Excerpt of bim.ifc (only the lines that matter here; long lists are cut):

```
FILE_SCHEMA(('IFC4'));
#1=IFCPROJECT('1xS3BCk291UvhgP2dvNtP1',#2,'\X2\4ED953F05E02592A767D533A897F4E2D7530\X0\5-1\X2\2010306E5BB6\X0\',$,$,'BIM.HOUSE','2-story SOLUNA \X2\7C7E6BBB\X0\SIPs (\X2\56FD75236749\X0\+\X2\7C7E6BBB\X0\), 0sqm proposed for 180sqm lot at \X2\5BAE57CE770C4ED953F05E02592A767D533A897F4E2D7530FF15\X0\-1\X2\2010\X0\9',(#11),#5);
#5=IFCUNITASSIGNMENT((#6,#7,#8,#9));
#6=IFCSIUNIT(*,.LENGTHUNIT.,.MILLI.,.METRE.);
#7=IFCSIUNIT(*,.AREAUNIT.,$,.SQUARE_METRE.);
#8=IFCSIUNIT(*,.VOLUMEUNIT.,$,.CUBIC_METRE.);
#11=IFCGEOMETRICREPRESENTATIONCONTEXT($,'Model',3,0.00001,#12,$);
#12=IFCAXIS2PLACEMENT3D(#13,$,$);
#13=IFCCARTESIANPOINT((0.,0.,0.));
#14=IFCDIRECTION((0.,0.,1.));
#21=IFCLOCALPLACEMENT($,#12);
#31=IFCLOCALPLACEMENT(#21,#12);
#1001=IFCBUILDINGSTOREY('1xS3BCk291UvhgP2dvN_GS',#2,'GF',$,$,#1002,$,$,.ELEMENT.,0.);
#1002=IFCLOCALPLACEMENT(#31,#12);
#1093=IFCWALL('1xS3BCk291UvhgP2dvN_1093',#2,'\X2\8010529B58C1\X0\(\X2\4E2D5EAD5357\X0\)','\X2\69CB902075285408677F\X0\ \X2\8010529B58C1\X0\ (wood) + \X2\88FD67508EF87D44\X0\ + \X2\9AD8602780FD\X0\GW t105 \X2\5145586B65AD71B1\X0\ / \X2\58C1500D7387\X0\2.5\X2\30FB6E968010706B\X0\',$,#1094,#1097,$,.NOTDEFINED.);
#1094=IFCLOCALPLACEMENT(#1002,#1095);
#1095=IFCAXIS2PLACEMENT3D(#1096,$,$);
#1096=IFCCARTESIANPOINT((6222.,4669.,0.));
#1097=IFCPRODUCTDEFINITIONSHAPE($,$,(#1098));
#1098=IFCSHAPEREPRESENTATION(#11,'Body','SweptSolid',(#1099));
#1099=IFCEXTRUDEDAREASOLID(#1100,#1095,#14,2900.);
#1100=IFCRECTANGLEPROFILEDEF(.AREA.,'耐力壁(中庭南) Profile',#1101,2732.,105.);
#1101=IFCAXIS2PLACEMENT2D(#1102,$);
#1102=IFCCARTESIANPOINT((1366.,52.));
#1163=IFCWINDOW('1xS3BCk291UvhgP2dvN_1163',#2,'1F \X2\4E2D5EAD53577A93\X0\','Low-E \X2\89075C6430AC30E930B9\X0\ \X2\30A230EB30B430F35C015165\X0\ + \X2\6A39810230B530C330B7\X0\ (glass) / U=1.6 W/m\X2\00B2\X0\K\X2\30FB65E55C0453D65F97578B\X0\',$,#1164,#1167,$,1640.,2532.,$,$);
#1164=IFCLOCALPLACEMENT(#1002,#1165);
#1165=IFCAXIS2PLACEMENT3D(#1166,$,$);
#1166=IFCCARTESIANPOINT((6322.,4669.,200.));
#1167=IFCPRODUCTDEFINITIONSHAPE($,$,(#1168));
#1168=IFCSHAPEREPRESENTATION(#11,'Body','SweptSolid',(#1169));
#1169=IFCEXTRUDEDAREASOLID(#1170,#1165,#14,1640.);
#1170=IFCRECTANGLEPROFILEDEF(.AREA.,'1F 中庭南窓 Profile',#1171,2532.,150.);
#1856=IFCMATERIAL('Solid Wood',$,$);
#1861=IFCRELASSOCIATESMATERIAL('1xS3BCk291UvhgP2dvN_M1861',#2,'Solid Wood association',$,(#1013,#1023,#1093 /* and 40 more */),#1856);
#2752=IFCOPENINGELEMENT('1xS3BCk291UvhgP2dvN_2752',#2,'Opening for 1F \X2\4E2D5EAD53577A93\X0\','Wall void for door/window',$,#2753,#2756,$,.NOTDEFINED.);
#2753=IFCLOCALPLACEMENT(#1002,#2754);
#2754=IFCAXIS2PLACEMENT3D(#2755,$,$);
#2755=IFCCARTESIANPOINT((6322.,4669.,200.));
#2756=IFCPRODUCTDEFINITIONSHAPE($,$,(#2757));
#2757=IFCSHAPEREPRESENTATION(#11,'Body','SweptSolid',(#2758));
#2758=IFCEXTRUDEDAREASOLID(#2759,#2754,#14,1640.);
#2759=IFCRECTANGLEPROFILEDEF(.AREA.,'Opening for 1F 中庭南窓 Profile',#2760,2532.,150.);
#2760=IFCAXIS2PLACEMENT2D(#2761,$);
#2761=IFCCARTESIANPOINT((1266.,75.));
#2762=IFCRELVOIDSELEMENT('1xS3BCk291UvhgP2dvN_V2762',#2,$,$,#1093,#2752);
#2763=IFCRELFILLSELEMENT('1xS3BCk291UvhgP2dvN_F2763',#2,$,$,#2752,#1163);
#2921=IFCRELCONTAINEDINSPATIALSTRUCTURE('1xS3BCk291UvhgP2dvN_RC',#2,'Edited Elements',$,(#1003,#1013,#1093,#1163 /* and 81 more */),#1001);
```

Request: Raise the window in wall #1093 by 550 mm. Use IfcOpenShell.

```python
import numpy as np
import ifcopenshell
import ifcopenshell.api.geometry
import ifcopenshell.util.placement
import ifcopenshell.util.unit

model = ifcopenshell.open("bim.ifc")
unit_scale = ifcopenshell.util.unit.calculate_unit_scale(model)

window = model.by_id(1163)
opening = window.FillsVoids[0].RelatingOpeningElement
dz = 0.55 / unit_scale

shift = np.array([0.0, 0.0, dz])
# The window is not placed relative to its opening, so move both.
for product in (opening, window):
    matrix = ifcopenshell.util.placement.get_local_placement(product.ObjectPlacement)
    matrix[:3, 3] += shift
    ifcopenshell.api.geometry.edit_object_placement(model, product=product, matrix=matrix, is_si=False)

print(f"moved by {dz * unit_scale:+.3f} m")

model.write("bim-out.ifc")
```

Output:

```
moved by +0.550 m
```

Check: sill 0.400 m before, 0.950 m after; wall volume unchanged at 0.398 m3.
